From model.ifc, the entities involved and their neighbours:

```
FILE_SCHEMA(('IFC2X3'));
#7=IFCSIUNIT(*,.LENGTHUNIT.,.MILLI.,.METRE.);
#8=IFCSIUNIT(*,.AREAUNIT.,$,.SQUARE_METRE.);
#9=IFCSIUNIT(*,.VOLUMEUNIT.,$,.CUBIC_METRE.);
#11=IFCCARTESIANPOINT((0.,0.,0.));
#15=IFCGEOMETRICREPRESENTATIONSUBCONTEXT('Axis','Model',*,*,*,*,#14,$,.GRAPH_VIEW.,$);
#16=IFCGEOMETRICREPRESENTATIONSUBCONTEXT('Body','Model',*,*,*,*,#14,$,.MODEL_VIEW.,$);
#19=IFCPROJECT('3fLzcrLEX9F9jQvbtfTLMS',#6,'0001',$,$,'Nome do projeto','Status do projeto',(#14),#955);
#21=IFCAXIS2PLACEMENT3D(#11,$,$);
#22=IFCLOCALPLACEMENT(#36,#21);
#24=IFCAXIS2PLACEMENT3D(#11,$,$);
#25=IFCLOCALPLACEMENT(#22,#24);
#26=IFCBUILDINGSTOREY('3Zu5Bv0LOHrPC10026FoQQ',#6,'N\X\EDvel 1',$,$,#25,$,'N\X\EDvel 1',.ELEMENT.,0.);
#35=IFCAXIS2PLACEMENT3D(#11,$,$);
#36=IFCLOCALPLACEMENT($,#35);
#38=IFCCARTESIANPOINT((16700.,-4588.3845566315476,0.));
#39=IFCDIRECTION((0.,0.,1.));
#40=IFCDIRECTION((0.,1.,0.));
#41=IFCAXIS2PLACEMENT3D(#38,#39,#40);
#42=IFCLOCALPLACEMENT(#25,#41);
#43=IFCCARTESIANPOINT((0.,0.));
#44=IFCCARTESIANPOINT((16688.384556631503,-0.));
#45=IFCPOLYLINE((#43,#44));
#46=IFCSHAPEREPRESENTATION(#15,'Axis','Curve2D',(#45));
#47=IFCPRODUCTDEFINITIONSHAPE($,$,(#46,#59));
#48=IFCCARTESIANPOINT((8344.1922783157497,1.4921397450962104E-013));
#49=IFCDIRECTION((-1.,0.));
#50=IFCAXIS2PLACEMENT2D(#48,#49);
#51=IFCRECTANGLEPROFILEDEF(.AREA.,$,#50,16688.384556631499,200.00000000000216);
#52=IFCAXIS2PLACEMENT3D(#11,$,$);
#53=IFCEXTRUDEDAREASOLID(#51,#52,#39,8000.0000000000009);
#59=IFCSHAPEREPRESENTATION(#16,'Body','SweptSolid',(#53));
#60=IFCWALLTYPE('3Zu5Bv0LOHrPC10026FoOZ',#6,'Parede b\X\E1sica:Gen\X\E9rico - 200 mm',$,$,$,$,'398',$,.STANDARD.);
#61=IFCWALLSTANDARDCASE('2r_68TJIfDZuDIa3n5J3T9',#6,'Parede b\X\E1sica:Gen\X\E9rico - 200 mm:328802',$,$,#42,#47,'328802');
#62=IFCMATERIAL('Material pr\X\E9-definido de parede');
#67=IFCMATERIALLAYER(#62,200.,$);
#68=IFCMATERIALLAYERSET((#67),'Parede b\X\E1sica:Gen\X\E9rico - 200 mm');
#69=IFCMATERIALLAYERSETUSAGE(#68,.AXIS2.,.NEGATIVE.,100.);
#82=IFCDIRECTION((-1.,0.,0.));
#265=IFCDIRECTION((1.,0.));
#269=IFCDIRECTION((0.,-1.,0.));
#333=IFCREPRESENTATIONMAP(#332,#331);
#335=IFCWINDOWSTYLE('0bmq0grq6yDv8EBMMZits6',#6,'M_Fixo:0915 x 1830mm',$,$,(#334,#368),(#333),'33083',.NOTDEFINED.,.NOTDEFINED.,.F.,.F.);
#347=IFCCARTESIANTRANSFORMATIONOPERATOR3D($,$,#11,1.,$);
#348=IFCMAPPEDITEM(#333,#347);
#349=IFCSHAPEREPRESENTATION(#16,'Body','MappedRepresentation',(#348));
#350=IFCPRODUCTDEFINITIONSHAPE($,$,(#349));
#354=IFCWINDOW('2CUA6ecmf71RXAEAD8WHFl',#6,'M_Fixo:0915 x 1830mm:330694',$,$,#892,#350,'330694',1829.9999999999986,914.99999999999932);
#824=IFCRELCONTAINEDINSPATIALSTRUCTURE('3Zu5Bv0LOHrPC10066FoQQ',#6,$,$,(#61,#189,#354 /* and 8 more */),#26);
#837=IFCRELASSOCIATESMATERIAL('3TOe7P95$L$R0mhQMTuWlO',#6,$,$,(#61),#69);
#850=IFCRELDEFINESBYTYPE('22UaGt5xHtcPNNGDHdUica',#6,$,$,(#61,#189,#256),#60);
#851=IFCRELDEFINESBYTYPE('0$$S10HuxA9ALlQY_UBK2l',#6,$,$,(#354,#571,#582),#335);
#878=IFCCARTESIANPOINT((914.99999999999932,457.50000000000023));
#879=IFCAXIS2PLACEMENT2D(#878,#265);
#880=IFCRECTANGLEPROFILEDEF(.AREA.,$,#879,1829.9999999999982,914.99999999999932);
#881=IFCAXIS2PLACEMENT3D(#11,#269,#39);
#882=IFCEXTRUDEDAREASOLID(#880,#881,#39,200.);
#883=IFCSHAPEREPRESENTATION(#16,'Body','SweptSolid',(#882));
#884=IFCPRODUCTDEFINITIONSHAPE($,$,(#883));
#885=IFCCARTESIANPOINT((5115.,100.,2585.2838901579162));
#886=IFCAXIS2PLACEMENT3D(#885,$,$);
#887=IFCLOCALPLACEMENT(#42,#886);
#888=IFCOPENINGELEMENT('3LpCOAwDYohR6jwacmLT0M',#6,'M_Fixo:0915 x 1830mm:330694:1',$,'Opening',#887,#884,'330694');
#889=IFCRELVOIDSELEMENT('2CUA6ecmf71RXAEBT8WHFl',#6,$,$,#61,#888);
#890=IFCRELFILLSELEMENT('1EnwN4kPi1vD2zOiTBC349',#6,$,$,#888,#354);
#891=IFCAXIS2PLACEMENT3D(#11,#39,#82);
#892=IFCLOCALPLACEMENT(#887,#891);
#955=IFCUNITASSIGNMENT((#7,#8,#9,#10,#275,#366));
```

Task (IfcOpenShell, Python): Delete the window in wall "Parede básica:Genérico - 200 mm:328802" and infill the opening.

```python
import ifcopenshell
import ifcopenshell.api.feature
import ifcopenshell.api.root
import ifcopenshell.geom
import ifcopenshell.util.shape

model = ifcopenshell.open("model.ifc")
settings = ifcopenshell.geom.settings()


def volume(element):
    """Net volume in cubic metres, openings subtracted."""
    shape = ifcopenshell.geom.create_shape(settings, element)
    return ifcopenshell.util.shape.get_volume(shape.geometry)


window = model.by_guid("2CUA6ecmf71RXAEAD8WHFl")
opening = window.FillsVoids[0].RelatingOpeningElement
wall = opening.VoidsElements[0].RelatingBuildingElement
before = volume(wall)

ifcopenshell.api.root.remove_product(model, product=window)
ifcopenshell.api.feature.remove_feature(model, feature=opening)

after = volume(wall)

print(f"wall volume {before:.3f} -> {after:.3f} m3")

model.write("model_v2.ifc")
```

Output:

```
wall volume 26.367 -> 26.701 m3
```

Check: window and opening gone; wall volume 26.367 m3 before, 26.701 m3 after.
